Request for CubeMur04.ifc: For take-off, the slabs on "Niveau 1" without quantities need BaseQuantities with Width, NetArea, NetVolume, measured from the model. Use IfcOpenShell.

First a look at what the model holds.

```python
import ifcopenshell
import ifcopenshell.util.element
import ifcopenshell.util.unit

model = ifcopenshell.open("CubeMur04.ifc")
print(model.schema)
for unit_type in ("LENGTHUNIT", "AREAUNIT", "VOLUMEUNIT"):
    print(unit_type, ifcopenshell.util.unit.calculate_unit_scale(model, unit_type))
storey = next(s for s in model.by_type("IfcBuildingStorey") if s.Name == "Niveau 1")
slabs = [e for e in ifcopenshell.util.element.get_decomposition(storey) if e.is_a("IfcSlab")]
for e in sorted(slabs, key=lambda e: e.id()):
    print(e.id(), e.is_a(), e.Name, list(ifcopenshell.util.element.get_psets(e, qtos_only=True)), sep=" | ")
```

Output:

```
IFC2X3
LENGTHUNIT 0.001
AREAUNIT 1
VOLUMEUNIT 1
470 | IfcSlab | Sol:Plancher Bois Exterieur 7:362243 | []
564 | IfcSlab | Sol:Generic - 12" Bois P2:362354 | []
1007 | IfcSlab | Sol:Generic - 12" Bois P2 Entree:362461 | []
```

```python
import ifcopenshell
import ifcopenshell.api.pset
import ifcopenshell.geom
import ifcopenshell.util.element
import ifcopenshell.util.shape
import ifcopenshell.util.unit

model = ifcopenshell.open("CubeMur04.ifc")
unit_scale = ifcopenshell.util.unit.calculate_unit_scale(model)
area_scale = ifcopenshell.util.unit.calculate_unit_scale(model, "AREAUNIT")
volume_scale = ifcopenshell.util.unit.calculate_unit_scale(model, "VOLUMEUNIT")
settings = ifcopenshell.geom.settings()

storey = next(s for s in model.by_type("IfcBuildingStorey") if s.Name == "Niveau 1")
slabs = [e for e in ifcopenshell.util.element.get_decomposition(storey) if e.is_a("IfcSlab")]

for e in sorted(slabs, key=lambda e: e.id()):
    if ifcopenshell.util.element.get_psets(e, qtos_only=True, should_inherit=False):
        continue
    # Geometry comes back in metres, in the element's own axes.
    shape = ifcopenshell.geom.create_shape(settings, e)
    values = {
        "Width": ifcopenshell.util.shape.get_z(shape.geometry) / unit_scale,
        "NetArea": ifcopenshell.util.shape.get_footprint_area(shape.geometry) / area_scale,
        "NetVolume": ifcopenshell.util.shape.get_volume(shape.geometry) / volume_scale,
    }
    qto = ifcopenshell.api.pset.add_qto(model, product=e, name="BaseQuantities")
    ifcopenshell.api.pset.edit_qto(model, qto=qto, properties=values)
    print(e.id(), {k: round(v, 3) for k, v in values.items()})

model.write("CubeMur04_edited.ifc")
```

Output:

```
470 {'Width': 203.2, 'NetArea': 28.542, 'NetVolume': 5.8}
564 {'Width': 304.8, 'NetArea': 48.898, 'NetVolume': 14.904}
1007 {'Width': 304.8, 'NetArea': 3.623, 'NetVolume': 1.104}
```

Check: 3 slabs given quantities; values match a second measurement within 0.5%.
